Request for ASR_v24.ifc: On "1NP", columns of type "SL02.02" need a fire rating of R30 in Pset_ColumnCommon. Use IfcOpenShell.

First a look at what the model holds.

```python
import ifcopenshell
import ifcopenshell.util.element

model = ifcopenshell.open("ASR_v24.ifc")
print(model.schema)
storey = next(s for s in model.by_type("IfcBuildingStorey") if s.Name == "1NP")
columns = [e for e in ifcopenshell.util.element.get_decomposition(storey) if e.is_a("IfcColumn")]
seen = {}
for e in columns:
    element_type = ifcopenshell.util.element.get_type(e)
    key = (element_type.Name if element_type != e and element_type else None, ifcopenshell.util.element.get_pset(e, "Pset_ColumnCommon", "FireRating"))
    seen[key] = seen.get(key, 0) + 1
for (name, value), count in sorted(seen.items(), key=str):
    print(count, "x", name, "|", value)
```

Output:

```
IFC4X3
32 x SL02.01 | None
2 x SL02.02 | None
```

```python
import ifcopenshell
import ifcopenshell.api.pset
import ifcopenshell.util.element

model = ifcopenshell.open("ASR_v24.ifc")

storey = next(s for s in model.by_type("IfcBuildingStorey") if s.Name == "1NP")
columns = [e for e in ifcopenshell.util.element.get_decomposition(storey) if e.is_a("IfcColumn")]

count = 0
for e in columns:
    element_type = ifcopenshell.util.element.get_type(e)
    if element_type in (None, e) or element_type.Name != "SL02.02":
        continue
    # add_pset returns the element's existing set when there is one.
    pset = ifcopenshell.api.pset.add_pset(model, product=e, name="Pset_ColumnCommon")
    ifcopenshell.api.pset.edit_pset(model, pset=pset, properties={"FireRating": "R30"})
    count += 1

print(count, "columns updated")

model.write("ASR_v24-out.ifc")
```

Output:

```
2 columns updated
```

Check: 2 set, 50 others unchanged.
